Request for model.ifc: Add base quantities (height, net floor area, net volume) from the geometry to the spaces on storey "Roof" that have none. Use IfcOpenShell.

First a look at what the model holds.

```python
import ifcopenshell
import ifcopenshell.util.element
import ifcopenshell.util.unit

model = ifcopenshell.open("model.ifc")
print(model.schema)
for unit_type in ("LENGTHUNIT", "AREAUNIT", "VOLUMEUNIT"):
    print(unit_type, ifcopenshell.util.unit.calculate_unit_scale(model, unit_type))
storey = next(s for s in model.by_type("IfcBuildingStorey") if s.Name == "Roof")
spaces = [e for e in ifcopenshell.util.element.get_decomposition(storey) if e.is_a("IfcSpace")]
for e in sorted(spaces, key=lambda e: e.id()):
    print(e.id(), e.is_a(), e.Name, list(ifcopenshell.util.element.get_psets(e, qtos_only=True)), sep=" | ")
```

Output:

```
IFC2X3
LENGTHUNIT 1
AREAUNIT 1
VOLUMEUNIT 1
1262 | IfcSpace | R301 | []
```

```python
import ifcopenshell
import ifcopenshell.api.pset
import ifcopenshell.geom
import ifcopenshell.util.element
import ifcopenshell.util.shape
import ifcopenshell.util.unit

model = ifcopenshell.open("model.ifc")
unit_scale = ifcopenshell.util.unit.calculate_unit_scale(model)
area_scale = ifcopenshell.util.unit.calculate_unit_scale(model, "AREAUNIT")
volume_scale = ifcopenshell.util.unit.calculate_unit_scale(model, "VOLUMEUNIT")
settings = ifcopenshell.geom.settings()

storey = next(s for s in model.by_type("IfcBuildingStorey") if s.Name == "Roof")
spaces = [e for e in ifcopenshell.util.element.get_decomposition(storey) if e.is_a("IfcSpace")]

for e in sorted(spaces, key=lambda e: e.id()):
    if ifcopenshell.util.element.get_psets(e, qtos_only=True, should_inherit=False):
        continue
    # Geometry comes back in metres, in the element's own axes.
    shape = ifcopenshell.geom.create_shape(settings, e)
    values = {
        "Height": ifcopenshell.util.shape.get_z(shape.geometry) / unit_scale,
        "NetFloorArea": ifcopenshell.util.shape.get_footprint_area(shape.geometry) / area_scale,
        "NetVolume": ifcopenshell.util.shape.get_volume(shape.geometry) / volume_scale,
    }
    qto = ifcopenshell.api.pset.add_qto(model, product=e, name="BaseQuantities")
    ifcopenshell.api.pset.edit_qto(model, qto=qto, properties=values)
    print(e.id(), {k: round(v, 3) for k, v in values.items()})

model.write("model_edited.ifc")
```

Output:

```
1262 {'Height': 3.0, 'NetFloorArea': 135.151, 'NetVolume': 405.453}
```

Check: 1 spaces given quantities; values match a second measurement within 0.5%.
